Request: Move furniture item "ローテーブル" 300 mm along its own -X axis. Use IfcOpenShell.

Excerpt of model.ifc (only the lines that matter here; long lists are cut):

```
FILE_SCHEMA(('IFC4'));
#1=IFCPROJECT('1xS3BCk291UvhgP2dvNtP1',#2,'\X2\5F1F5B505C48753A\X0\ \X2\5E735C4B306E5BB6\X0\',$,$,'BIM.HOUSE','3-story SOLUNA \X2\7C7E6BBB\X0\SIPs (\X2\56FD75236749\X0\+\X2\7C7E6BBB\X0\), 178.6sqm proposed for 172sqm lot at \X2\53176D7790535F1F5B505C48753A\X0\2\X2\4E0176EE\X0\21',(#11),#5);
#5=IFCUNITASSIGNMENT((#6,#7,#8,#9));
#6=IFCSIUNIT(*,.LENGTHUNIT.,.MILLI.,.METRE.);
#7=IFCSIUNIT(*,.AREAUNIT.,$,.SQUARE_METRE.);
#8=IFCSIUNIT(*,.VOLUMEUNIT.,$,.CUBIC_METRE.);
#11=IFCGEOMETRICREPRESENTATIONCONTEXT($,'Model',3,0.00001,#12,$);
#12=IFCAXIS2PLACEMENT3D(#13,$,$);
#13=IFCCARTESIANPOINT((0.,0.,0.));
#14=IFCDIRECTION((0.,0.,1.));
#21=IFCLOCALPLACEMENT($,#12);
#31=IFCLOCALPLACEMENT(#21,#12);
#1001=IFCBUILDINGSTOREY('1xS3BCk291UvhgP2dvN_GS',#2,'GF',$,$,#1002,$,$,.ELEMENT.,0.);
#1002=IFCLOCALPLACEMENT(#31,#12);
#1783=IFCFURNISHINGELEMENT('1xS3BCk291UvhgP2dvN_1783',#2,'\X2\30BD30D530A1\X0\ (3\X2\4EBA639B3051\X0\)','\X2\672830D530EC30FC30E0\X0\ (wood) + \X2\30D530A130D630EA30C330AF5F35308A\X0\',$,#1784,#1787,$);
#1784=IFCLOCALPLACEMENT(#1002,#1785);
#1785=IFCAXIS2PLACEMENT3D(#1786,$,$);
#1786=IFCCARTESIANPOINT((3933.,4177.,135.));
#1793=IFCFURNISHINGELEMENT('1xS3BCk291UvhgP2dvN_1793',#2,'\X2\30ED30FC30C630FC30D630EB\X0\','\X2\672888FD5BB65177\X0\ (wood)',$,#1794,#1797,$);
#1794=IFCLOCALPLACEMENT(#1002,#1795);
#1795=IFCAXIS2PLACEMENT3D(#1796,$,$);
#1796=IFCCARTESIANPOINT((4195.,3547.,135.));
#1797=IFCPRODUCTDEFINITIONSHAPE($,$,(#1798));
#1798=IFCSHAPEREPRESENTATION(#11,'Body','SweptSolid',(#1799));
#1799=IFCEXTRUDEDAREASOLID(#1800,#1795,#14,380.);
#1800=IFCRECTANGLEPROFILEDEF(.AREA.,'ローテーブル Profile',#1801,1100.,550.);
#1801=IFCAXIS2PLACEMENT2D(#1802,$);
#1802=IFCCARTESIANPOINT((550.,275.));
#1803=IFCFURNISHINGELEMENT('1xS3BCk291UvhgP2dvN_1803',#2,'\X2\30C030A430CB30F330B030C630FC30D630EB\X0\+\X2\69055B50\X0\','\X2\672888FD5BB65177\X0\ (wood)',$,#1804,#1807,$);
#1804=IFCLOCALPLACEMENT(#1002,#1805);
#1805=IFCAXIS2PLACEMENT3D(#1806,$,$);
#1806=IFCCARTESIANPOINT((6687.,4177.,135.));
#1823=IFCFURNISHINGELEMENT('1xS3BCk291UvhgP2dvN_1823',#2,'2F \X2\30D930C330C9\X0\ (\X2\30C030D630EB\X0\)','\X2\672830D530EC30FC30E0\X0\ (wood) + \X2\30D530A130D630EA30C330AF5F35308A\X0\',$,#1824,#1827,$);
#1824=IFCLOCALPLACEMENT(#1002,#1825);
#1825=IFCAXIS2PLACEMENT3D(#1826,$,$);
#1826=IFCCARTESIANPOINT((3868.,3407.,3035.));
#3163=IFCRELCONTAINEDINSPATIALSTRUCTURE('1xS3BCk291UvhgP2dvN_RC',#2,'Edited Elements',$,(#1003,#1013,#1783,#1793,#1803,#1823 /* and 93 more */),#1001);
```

```python
import ifcopenshell
import ifcopenshell.api.geometry
import ifcopenshell.util.placement

model = ifcopenshell.open("model.ifc")

item = model.by_id(1793)
matrix = ifcopenshell.util.placement.get_local_placement(item.ObjectPlacement)
matrix[:3, 3] -= matrix[:3, 0] * 300.0
ifcopenshell.api.geometry.edit_object_placement(model, product=item, matrix=matrix, is_si=False)

print(ifcopenshell.util.placement.get_local_placement(item.ObjectPlacement).round(3) + 0.0)

model.write("model_rev.ifc")
```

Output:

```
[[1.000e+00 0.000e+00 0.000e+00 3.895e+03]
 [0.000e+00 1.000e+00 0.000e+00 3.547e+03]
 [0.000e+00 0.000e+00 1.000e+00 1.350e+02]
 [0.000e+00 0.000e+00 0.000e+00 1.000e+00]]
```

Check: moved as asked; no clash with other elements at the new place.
